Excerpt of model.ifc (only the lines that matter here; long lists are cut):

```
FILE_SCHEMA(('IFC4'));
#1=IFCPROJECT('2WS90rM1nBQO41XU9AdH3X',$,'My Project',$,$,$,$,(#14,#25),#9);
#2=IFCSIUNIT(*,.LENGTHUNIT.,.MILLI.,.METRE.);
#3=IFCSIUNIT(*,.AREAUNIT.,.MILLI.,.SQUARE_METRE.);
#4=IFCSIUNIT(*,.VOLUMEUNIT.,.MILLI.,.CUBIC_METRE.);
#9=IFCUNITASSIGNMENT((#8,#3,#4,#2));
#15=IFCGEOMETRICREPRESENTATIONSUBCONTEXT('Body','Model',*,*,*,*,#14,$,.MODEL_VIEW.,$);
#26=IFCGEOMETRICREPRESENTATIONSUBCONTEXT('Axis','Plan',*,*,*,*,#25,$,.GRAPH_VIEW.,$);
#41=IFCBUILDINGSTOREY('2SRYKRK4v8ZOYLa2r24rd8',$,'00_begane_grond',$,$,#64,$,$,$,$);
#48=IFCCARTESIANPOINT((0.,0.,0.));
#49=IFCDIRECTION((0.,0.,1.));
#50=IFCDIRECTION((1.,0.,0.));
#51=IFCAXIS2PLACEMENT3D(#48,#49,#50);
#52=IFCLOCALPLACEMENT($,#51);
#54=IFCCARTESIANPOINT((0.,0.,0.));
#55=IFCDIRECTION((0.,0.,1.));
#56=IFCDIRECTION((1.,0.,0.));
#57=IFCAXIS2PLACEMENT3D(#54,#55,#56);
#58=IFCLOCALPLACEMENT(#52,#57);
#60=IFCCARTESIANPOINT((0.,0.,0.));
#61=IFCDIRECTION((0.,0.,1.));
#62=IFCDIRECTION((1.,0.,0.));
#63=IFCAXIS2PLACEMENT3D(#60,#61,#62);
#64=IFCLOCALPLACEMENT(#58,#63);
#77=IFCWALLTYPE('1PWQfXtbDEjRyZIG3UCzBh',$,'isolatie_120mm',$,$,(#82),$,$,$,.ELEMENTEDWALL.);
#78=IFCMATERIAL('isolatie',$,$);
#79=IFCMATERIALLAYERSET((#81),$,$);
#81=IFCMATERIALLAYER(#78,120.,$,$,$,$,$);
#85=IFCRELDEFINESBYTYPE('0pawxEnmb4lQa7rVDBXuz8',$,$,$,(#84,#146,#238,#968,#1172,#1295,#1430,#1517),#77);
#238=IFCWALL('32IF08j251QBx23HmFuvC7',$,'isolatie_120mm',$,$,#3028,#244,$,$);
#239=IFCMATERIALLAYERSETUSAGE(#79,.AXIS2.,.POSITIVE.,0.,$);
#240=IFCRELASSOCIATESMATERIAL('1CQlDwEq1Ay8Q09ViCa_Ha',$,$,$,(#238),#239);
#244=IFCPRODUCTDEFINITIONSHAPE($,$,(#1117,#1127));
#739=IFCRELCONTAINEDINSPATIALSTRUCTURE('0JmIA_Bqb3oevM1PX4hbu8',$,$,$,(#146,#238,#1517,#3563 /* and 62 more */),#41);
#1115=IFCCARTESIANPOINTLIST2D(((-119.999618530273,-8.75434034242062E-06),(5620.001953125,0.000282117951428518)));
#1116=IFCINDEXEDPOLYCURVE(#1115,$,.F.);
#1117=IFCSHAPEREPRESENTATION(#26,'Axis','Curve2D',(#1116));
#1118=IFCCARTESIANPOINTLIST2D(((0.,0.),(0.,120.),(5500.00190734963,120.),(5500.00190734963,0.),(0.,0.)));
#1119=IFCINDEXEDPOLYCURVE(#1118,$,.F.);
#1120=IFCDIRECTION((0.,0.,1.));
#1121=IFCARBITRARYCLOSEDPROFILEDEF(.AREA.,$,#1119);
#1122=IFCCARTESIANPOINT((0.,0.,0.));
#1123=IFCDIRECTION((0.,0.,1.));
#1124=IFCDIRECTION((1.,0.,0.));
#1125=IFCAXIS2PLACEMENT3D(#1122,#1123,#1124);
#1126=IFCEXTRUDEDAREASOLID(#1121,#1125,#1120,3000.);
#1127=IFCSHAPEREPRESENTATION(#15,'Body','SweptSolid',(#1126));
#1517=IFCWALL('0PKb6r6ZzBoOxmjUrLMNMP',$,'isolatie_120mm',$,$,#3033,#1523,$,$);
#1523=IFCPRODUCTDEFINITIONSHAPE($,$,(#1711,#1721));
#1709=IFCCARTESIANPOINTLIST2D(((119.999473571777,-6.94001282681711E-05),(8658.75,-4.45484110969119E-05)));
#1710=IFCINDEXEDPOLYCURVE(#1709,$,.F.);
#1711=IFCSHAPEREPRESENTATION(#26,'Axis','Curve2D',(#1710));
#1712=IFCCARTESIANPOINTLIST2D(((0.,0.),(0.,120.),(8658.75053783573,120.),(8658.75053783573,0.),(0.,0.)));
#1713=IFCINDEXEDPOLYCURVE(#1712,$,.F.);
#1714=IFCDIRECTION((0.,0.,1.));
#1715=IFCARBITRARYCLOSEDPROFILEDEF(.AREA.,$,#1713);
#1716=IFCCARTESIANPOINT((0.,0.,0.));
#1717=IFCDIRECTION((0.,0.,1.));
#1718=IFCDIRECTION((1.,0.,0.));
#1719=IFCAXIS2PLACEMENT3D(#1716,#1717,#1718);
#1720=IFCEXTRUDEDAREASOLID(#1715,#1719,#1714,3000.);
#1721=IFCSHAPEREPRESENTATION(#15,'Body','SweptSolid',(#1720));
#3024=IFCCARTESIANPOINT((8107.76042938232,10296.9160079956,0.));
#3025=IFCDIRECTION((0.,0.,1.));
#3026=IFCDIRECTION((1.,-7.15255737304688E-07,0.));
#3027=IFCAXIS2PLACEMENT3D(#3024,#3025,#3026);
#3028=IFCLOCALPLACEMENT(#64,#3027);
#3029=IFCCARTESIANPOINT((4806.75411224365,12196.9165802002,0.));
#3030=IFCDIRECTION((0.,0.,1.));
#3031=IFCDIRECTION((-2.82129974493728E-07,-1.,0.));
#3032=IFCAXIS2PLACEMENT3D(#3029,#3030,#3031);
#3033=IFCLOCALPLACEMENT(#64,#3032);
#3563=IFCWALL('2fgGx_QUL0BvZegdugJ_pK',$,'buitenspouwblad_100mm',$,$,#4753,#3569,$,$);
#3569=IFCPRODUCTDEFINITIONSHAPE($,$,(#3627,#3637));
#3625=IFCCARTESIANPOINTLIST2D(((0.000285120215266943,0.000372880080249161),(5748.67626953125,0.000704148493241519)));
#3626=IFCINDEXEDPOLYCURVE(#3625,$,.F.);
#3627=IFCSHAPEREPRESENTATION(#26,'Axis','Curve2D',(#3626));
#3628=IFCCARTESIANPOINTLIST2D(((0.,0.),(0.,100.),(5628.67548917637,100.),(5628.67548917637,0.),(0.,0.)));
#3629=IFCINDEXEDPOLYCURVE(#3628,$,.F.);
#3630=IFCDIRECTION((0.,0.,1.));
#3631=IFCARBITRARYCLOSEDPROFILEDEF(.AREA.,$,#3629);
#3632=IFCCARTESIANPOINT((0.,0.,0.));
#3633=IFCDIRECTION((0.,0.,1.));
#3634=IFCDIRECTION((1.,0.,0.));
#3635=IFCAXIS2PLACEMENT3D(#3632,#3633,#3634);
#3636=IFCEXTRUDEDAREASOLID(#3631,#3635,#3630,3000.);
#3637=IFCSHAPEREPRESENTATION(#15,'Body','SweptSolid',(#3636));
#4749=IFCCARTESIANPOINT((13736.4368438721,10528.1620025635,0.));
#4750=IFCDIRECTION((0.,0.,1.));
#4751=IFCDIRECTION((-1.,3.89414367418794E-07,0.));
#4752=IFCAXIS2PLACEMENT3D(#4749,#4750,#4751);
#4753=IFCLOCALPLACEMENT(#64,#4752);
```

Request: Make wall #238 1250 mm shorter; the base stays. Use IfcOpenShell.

```python
import ifcopenshell
import ifcopenshell.geom
import ifcopenshell.util.representation
import ifcopenshell.util.shape
import ifcopenshell.util.unit

model = ifcopenshell.open("model.ifc")
unit_scale = ifcopenshell.util.unit.calculate_unit_scale(model)
settings = ifcopenshell.geom.settings()


def volume(element):
    """Net volume in cubic metres, openings subtracted."""
    shape = ifcopenshell.geom.create_shape(settings, element)
    return ifcopenshell.util.shape.get_volume(shape.geometry)


wall = model.by_id(238)
before = volume(wall)

body = ifcopenshell.util.representation.get_representation(wall, "Model", "Body")
solid = body.Items[0]
old_height = solid.Depth
solid.Depth -= 1.25 / unit_scale
after = volume(wall)

print(f"height {old_height:g} -> {solid.Depth:g}, volume {before:.3f} -> {after:.3f} m3")

model.write("model_rev.ifc")
```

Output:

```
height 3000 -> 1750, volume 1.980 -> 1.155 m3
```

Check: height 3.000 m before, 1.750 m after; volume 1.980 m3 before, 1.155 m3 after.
